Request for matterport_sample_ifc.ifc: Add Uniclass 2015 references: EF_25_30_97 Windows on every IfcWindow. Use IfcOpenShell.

First a look at what the model holds.

```python
import ifcopenshell

model = ifcopenshell.open("matterport_sample_ifc.ifc")
print(model.schema)
print("classifications:", [c.Name for c in model.by_type("IfcClassification")])
for ifc_class in ("IfcDoor", "IfcRoof", "IfcStair", "IfcWall", "IfcWindow"):
    print(ifc_class, len(model.by_type(ifc_class)))
```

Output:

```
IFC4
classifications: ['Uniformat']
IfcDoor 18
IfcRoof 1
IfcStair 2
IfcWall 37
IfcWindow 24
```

```python
import ifcopenshell
import ifcopenshell.api.classification

model = ifcopenshell.open("matterport_sample_ifc.ifc")

system = ifcopenshell.api.classification.add_classification(model, classification="Uniclass 2015")

codes = {
    "IfcWindow": ("EF_25_30_97", "Windows"),
}
for ifc_class, (code, name) in codes.items():
    products = model.by_type(ifc_class)
    ifcopenshell.api.classification.add_reference(
        model, products=products, classification=system, identification=code, name=name
    )
    print(code, len(products))

model.write("matterport_sample_ifc-out.ifc")
```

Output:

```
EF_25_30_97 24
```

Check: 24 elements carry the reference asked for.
